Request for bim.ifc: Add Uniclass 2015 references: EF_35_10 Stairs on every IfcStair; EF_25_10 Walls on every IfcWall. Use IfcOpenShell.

First a look at what the model holds.

```python
import ifcopenshell

model = ifcopenshell.open("bim.ifc")
print(model.schema)
print("classifications:", [c.Name for c in model.by_type("IfcClassification")])
for ifc_class in ("IfcDoor", "IfcRoof", "IfcStair", "IfcWall", "IfcWindow"):
    print(ifc_class, len(model.by_type(ifc_class)))
```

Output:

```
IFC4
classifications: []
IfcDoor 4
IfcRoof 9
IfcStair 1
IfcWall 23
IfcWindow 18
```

```python
import ifcopenshell
import ifcopenshell.api.classification

model = ifcopenshell.open("bim.ifc")

system = ifcopenshell.api.classification.add_classification(model, classification="Uniclass 2015")

codes = {
    "IfcStair": ("EF_35_10", "Stairs"),
    "IfcWall": ("EF_25_10", "Walls"),
}
for ifc_class, (code, name) in codes.items():
    products = model.by_type(ifc_class)
    ifcopenshell.api.classification.add_reference(
        model, products=products, classification=system, identification=code, name=name
    )
    print(code, len(products))

model.write("bim_rev.ifc")
```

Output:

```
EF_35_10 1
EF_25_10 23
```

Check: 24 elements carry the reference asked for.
